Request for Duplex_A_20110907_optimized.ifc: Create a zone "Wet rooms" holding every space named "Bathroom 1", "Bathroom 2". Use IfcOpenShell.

First a look at what the model holds.

```python
import ifcopenshell

model = ifcopenshell.open("Duplex_A_20110907_optimized.ifc")
print(model.schema)
seen = {}
for space in model.by_type("IfcSpace"):
    seen[space.LongName] = seen.get(space.LongName, 0) + 1
for name, count in sorted(seen.items(), key=str):
    print(count, "x", name)
print("zones:", [z.Name for z in model.by_type("IfcZone")][:20])
```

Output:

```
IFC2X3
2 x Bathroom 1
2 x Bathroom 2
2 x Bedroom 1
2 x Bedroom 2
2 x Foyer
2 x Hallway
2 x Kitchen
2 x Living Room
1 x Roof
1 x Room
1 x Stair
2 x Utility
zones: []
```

```python
import ifcopenshell
import ifcopenshell.api.group
import ifcopenshell.api.root

model = ifcopenshell.open("Duplex_A_20110907_optimized.ifc")

names = {"Bathroom 1", "Bathroom 2"}
spaces = [s for s in model.by_type("IfcSpace") if s.LongName in names]

zone = ifcopenshell.api.root.create_entity(model, ifc_class="IfcZone", name="Wet rooms")
ifcopenshell.api.group.assign_group(model, products=spaces, group=zone)
print(len(spaces), "spaces in", zone.Name)

model.write("Duplex_A_20110907_optimized_updated.ifc")
```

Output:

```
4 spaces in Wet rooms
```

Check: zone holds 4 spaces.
